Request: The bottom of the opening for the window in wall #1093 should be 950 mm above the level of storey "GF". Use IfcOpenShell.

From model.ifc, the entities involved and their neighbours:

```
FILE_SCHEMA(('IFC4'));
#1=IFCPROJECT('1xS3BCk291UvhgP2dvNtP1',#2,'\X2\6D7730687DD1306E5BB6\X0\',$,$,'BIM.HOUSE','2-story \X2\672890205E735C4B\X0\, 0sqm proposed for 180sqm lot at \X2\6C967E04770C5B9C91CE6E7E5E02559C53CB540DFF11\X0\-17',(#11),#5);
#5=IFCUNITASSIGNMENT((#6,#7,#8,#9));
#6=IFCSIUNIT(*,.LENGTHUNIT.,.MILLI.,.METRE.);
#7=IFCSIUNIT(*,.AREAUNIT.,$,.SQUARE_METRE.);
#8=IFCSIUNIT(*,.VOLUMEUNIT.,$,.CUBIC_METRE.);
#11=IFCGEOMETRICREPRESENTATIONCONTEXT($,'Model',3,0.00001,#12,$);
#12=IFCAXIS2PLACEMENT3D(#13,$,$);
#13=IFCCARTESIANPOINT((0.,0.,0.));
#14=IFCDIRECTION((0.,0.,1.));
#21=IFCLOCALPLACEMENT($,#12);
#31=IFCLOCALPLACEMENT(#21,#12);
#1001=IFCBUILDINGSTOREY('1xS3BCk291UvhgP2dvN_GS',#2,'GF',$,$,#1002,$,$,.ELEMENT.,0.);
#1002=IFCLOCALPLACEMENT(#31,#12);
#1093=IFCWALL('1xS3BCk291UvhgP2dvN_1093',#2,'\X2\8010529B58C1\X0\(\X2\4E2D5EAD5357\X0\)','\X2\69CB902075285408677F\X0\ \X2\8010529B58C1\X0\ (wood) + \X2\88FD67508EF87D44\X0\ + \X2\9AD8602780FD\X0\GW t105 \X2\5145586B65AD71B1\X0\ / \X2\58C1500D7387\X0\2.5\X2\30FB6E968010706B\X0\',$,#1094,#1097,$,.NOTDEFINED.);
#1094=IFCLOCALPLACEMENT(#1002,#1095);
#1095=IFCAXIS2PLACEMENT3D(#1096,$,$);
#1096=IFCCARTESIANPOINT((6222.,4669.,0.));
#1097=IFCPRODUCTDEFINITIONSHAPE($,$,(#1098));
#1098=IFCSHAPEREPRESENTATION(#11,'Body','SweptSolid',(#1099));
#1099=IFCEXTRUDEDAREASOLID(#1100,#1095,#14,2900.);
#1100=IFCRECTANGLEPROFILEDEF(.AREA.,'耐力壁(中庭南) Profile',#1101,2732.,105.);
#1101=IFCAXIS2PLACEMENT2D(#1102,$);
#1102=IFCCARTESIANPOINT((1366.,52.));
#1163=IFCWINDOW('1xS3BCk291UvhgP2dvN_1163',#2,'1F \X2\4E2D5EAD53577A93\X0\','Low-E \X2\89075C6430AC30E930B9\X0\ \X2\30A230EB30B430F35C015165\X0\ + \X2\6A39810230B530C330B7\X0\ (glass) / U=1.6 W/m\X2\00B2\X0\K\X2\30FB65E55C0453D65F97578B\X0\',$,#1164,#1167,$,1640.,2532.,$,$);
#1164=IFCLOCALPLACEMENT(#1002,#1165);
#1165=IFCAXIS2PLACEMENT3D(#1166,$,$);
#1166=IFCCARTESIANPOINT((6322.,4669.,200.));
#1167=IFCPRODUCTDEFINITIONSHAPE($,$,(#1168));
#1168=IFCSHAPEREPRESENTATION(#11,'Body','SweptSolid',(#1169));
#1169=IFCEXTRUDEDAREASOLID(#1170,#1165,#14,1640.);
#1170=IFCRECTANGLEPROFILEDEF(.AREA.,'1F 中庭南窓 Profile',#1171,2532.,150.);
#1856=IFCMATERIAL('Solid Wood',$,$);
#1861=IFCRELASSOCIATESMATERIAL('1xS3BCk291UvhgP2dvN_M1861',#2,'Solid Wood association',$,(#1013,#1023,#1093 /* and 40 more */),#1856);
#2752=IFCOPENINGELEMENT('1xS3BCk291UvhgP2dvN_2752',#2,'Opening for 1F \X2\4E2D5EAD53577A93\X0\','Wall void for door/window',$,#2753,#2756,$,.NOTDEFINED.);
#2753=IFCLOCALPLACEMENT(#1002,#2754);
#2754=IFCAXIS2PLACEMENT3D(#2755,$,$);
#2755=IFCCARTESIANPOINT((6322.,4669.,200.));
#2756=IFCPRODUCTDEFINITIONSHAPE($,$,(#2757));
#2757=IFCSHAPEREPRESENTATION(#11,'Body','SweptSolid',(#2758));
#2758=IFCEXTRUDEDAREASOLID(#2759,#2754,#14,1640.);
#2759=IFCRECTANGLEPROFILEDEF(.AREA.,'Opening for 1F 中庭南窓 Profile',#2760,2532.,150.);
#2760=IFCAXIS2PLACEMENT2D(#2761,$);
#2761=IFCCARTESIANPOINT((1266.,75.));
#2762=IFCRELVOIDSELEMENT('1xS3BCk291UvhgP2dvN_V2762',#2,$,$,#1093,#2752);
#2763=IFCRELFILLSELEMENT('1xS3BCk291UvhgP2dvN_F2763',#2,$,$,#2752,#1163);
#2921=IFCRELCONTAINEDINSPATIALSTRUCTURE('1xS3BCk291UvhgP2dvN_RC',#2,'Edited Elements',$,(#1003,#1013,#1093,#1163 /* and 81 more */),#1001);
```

```python
import numpy as np
import ifcopenshell
import ifcopenshell.api.geometry
import ifcopenshell.geom
import ifcopenshell.util.element
import ifcopenshell.util.placement
import ifcopenshell.util.shape
import ifcopenshell.util.unit

model = ifcopenshell.open("model.ifc")
unit_scale = ifcopenshell.util.unit.calculate_unit_scale(model)

window = model.by_id(1163)
opening = window.FillsVoids[0].RelatingOpeningElement
storey = ifcopenshell.util.element.get_container(window, ifc_class="IfcBuildingStorey")
level = ifcopenshell.util.placement.get_local_placement(storey.ObjectPlacement)[2, 3]

# The opening's origin need not be at the sill, so measure its lowest point.
shape = ifcopenshell.geom.create_shape(ifcopenshell.geom.settings(), opening)
bottom = ifcopenshell.util.shape.get_shape_bottom_elevation(shape, shape.geometry) / unit_scale
dz = level + 950.0 - bottom

shift = np.array([0.0, 0.0, dz])
# The window is not placed relative to its opening, so move both.
for product in (opening, window):
    matrix = ifcopenshell.util.placement.get_local_placement(product.ObjectPlacement)
    matrix[:3, 3] += shift
    ifcopenshell.api.geometry.edit_object_placement(model, product=product, matrix=matrix, is_si=False)

print(f"moved by {dz * unit_scale:+.3f} m")

model.write("model-out.ifc")
```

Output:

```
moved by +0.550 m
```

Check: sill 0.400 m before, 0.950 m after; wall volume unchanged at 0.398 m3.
